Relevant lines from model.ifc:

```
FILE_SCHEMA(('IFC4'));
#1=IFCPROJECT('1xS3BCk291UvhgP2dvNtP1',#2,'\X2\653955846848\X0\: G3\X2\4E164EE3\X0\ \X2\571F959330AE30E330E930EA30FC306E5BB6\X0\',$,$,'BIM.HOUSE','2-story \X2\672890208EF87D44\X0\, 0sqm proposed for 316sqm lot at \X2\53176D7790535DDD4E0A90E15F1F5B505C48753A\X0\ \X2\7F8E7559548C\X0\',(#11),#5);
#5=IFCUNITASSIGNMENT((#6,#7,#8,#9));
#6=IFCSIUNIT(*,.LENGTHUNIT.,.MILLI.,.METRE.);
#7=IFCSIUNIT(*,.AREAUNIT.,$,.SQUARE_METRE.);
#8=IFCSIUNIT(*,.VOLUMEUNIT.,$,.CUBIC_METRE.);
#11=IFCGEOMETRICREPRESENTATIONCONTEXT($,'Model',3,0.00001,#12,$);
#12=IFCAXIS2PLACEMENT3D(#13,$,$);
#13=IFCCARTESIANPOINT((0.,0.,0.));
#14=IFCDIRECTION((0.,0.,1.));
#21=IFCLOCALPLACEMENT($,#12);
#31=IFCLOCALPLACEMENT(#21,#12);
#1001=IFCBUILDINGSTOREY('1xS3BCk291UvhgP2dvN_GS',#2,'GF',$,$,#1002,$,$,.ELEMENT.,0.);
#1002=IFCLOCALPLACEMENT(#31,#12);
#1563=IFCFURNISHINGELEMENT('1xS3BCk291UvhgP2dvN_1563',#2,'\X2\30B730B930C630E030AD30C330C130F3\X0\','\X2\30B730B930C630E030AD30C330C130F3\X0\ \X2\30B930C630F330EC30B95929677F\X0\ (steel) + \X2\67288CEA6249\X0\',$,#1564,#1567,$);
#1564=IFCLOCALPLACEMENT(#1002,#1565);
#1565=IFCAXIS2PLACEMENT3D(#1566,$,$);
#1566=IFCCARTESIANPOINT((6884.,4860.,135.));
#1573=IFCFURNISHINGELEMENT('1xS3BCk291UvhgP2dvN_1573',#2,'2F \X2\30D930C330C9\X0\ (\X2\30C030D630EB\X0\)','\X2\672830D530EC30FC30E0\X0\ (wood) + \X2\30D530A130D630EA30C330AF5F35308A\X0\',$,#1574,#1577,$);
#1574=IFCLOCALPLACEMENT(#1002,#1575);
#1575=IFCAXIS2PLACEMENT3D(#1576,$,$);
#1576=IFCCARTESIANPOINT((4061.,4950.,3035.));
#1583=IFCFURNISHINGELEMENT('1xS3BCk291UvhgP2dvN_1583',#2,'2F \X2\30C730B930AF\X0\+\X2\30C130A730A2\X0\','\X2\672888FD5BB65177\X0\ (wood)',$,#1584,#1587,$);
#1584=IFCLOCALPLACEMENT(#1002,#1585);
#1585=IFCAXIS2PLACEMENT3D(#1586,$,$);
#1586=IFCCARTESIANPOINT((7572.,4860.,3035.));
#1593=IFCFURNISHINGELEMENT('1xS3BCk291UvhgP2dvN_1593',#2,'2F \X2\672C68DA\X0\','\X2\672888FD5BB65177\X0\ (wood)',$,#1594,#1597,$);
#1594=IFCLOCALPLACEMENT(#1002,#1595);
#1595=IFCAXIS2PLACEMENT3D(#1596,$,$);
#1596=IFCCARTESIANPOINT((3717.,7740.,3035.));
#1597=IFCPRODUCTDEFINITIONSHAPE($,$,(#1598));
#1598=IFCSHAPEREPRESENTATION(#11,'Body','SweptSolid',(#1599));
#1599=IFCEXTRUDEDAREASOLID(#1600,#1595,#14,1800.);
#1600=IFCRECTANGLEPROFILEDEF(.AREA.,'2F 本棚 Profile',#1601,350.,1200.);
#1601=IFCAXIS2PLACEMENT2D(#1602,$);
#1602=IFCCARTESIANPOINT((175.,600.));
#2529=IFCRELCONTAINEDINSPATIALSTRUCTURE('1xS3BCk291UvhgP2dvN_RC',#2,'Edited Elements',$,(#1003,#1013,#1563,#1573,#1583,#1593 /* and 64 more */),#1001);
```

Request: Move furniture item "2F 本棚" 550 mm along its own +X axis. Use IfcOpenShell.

```python
import ifcopenshell
import ifcopenshell.api.geometry
import ifcopenshell.util.placement
import ifcopenshell.util.unit

model = ifcopenshell.open("model.ifc")
unit_scale = ifcopenshell.util.unit.calculate_unit_scale(model)

item = model.by_guid("1xS3BCk291UvhgP2dvN_1593")
matrix = ifcopenshell.util.placement.get_local_placement(item.ObjectPlacement)
matrix[:3, 3] += matrix[:3, 0] * 0.55 / unit_scale
ifcopenshell.api.geometry.edit_object_placement(model, product=item, matrix=matrix, is_si=False)

print(ifcopenshell.util.placement.get_local_placement(item.ObjectPlacement).round(3) + 0.0)

model.write("model_rev.ifc")
```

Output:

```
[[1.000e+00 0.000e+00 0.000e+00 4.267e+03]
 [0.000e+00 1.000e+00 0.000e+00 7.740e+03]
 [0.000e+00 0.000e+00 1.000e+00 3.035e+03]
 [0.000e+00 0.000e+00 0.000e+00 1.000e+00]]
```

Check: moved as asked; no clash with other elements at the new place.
